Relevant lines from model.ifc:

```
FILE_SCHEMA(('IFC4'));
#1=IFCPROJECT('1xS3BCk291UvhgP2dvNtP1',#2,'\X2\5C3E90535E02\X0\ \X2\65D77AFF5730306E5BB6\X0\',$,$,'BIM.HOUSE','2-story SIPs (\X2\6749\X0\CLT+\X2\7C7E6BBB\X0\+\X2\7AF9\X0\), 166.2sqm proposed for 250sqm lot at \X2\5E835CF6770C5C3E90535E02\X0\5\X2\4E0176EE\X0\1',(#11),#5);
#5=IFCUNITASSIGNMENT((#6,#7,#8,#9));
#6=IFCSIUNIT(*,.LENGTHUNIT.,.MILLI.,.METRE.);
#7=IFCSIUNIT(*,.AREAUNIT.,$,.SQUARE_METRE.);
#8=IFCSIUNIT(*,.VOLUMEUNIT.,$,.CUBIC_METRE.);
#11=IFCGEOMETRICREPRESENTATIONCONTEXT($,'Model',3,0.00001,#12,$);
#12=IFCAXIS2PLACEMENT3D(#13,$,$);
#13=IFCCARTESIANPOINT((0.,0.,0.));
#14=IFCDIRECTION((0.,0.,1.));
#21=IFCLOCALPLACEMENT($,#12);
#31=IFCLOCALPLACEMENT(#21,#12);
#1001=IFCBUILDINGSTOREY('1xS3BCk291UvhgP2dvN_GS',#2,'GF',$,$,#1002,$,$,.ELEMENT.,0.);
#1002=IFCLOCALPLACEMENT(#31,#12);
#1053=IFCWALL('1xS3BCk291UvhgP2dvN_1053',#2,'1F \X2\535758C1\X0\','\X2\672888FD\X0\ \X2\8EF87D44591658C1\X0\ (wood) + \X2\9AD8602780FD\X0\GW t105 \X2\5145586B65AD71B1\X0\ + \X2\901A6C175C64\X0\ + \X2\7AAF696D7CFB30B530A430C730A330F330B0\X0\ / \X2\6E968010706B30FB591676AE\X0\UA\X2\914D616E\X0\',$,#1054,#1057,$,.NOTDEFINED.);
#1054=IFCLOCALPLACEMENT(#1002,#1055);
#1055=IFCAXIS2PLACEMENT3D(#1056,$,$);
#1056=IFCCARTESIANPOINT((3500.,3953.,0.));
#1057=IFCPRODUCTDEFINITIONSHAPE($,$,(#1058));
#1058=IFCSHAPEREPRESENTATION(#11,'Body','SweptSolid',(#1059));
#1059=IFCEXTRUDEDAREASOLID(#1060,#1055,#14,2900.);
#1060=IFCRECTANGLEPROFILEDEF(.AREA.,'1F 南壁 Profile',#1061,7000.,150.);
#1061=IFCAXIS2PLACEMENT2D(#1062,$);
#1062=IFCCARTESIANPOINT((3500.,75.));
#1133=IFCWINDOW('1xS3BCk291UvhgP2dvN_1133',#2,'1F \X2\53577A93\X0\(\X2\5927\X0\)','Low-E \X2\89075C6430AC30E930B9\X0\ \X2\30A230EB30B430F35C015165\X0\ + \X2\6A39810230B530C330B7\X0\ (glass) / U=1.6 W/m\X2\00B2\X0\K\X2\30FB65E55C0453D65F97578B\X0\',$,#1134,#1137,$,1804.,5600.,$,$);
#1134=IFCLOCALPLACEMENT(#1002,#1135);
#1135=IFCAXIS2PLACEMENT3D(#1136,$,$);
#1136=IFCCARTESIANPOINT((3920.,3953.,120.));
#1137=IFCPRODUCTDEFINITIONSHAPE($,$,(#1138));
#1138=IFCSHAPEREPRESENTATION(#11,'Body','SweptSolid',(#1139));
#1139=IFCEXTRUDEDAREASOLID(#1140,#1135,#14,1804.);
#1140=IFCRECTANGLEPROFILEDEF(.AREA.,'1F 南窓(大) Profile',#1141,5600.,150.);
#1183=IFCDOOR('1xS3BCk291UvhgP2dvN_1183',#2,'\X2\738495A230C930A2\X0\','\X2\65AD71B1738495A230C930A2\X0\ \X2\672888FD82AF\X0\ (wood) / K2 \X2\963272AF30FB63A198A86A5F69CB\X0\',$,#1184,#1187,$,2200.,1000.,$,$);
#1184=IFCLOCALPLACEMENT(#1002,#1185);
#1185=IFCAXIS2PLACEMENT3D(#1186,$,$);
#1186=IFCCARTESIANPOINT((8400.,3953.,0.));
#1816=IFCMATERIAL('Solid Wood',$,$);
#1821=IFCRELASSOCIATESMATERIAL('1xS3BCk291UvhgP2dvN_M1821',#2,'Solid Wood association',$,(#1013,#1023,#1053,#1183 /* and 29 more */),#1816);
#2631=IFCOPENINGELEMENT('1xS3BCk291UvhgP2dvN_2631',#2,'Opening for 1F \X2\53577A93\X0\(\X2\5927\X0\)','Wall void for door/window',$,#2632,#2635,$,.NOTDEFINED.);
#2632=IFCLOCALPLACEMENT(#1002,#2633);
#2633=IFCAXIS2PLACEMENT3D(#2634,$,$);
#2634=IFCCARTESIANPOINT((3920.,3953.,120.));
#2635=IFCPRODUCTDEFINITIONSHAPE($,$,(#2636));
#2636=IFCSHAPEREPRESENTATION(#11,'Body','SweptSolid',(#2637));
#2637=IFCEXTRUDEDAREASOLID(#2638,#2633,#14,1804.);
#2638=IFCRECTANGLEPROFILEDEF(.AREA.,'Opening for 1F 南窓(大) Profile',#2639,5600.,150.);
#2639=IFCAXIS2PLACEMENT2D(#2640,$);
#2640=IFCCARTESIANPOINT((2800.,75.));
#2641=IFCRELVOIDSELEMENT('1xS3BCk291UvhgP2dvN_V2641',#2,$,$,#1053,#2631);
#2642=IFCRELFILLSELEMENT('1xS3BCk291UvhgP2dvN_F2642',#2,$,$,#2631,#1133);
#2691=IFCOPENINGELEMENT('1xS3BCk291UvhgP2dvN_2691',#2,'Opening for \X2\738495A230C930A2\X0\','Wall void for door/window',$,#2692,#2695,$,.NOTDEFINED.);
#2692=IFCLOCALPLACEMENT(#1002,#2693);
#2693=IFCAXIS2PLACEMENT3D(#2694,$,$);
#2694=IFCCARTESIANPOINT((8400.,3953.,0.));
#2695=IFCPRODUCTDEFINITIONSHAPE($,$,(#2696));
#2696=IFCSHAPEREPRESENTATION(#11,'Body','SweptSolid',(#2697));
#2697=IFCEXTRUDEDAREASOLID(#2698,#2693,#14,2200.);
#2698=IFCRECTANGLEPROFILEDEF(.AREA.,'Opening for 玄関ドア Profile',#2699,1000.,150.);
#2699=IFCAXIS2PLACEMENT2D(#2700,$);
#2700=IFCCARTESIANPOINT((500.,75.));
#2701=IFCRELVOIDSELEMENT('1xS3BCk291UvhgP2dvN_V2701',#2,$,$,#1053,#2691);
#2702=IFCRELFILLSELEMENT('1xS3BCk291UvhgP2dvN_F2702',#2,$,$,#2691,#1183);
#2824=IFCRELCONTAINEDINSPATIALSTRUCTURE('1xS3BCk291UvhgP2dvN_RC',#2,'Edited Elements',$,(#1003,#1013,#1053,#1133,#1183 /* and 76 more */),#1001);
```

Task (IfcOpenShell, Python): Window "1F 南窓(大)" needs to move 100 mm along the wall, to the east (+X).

```python
import ifcopenshell
import ifcopenshell.api.geometry
import ifcopenshell.util.placement

model = ifcopenshell.open("model.ifc")

window = model.by_id(1133)
opening = window.FillsVoids[0].RelatingOpeningElement
wall = opening.VoidsElements[0].RelatingBuildingElement

wall_matrix = ifcopenshell.util.placement.get_local_placement(wall.ObjectPlacement)
shift = wall_matrix[:3, 0] * 100.0
before = ifcopenshell.util.placement.get_local_placement(window.ObjectPlacement)[:3, 3].copy()

# The window is not placed relative to its opening, so move both.
for product in (opening, window):
    matrix = ifcopenshell.util.placement.get_local_placement(product.ObjectPlacement)
    matrix[:3, 3] += shift
    ifcopenshell.api.geometry.edit_object_placement(model, product=product, matrix=matrix, is_si=False)

after = ifcopenshell.util.placement.get_local_placement(window.ObjectPlacement)[:3, 3]
print("window moved by", (after - before).round(3) + 0.0)

model.write("model_rev.ifc")
```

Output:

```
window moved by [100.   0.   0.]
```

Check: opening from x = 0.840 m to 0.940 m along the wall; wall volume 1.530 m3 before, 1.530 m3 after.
